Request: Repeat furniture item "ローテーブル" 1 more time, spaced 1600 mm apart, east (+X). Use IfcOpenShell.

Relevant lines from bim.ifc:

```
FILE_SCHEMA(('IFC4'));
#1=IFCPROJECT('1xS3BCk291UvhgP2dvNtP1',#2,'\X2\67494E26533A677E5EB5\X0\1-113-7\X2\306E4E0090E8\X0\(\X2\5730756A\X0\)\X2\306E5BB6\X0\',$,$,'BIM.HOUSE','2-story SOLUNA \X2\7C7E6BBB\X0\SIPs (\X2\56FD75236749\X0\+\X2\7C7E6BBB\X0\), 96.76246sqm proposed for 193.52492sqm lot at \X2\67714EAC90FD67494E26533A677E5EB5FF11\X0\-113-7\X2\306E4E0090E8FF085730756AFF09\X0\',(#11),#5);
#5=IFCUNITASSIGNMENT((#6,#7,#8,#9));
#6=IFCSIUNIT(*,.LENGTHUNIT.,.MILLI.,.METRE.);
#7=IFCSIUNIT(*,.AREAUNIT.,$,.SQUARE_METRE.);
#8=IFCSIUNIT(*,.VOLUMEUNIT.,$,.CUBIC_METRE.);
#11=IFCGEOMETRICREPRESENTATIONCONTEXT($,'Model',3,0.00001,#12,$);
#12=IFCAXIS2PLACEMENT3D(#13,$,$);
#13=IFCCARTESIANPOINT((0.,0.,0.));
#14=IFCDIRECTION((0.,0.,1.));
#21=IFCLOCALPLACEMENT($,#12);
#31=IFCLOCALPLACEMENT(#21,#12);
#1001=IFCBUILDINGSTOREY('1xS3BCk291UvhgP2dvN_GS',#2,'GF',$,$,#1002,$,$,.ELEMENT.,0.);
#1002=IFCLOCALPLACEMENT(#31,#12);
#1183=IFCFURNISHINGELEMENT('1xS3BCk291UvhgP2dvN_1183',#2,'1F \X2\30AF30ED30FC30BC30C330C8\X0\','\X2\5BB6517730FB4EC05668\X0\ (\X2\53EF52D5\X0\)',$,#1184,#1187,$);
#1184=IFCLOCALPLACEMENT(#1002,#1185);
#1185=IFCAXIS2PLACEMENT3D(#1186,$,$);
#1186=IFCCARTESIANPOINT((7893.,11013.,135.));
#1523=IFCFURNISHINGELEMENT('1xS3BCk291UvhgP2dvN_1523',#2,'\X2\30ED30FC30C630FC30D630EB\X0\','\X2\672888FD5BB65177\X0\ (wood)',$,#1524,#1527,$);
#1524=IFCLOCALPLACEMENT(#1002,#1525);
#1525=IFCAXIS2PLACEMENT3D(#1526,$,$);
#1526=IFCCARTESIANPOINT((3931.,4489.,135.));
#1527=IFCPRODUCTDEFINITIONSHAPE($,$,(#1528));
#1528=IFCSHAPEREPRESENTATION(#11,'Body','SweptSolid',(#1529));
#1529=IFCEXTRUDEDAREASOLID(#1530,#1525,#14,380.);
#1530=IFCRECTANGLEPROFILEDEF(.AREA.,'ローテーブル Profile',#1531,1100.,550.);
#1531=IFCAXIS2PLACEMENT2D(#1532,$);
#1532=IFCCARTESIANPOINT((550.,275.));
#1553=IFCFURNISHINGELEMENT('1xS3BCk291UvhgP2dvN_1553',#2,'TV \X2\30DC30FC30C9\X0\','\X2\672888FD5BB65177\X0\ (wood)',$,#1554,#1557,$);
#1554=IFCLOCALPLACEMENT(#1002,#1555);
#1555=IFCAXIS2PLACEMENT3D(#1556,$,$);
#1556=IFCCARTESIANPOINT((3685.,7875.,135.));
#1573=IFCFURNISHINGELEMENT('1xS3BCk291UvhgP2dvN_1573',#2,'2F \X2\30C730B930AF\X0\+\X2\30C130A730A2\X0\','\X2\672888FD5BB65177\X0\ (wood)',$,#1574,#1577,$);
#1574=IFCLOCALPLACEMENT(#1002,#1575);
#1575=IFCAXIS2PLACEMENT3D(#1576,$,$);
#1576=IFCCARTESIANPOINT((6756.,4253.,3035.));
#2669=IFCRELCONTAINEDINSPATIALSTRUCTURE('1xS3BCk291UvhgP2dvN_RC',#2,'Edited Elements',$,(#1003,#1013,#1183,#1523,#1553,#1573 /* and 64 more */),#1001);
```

```python
import numpy as np
import ifcopenshell
import ifcopenshell.api.geometry
import ifcopenshell.api.root
import ifcopenshell.util.element
import ifcopenshell.util.placement
import ifcopenshell.util.unit

model = ifcopenshell.open("bim.ifc")
unit_scale = ifcopenshell.util.unit.calculate_unit_scale(model)


def reuse_history(source, copy):
    """copy_class also copies each property set's owner history, people and application; keep the originals."""
    for rel in copy.IsDefinedBy:
        if rel.is_a("IfcRelDefinesByProperties") and (history := rel.RelatingPropertyDefinition.OwnerHistory):
            rel.RelatingPropertyDefinition.OwnerHistory = source.OwnerHistory
            ifcopenshell.util.element.remove_deep2(model, history)


source = model.by_guid("1xS3BCk291UvhgP2dvN_1523")
base = ifcopenshell.util.placement.get_local_placement(source.ObjectPlacement)
step = np.array([1.0, 0.0, 0.0]) * 1.6 / unit_scale

for i in range(1, 2):
    copy = ifcopenshell.api.root.copy_class(model, product=source)
    copy.Representation = ifcopenshell.util.element.copy_deep(
        model, source.Representation, exclude=["IfcGeometricRepresentationContext", "IfcRepresentationMap"]
    )
    reuse_history(source, copy)
    matrix = base.copy()
    matrix[:3, 3] += i * step
    print("added at", matrix[:3, 3].round(3) + 0.0)
    ifcopenshell.api.geometry.edit_object_placement(model, product=copy, matrix=matrix, is_si=False)

model.write("bim_v2.ifc")
```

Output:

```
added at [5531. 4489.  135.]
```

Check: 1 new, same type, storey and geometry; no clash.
